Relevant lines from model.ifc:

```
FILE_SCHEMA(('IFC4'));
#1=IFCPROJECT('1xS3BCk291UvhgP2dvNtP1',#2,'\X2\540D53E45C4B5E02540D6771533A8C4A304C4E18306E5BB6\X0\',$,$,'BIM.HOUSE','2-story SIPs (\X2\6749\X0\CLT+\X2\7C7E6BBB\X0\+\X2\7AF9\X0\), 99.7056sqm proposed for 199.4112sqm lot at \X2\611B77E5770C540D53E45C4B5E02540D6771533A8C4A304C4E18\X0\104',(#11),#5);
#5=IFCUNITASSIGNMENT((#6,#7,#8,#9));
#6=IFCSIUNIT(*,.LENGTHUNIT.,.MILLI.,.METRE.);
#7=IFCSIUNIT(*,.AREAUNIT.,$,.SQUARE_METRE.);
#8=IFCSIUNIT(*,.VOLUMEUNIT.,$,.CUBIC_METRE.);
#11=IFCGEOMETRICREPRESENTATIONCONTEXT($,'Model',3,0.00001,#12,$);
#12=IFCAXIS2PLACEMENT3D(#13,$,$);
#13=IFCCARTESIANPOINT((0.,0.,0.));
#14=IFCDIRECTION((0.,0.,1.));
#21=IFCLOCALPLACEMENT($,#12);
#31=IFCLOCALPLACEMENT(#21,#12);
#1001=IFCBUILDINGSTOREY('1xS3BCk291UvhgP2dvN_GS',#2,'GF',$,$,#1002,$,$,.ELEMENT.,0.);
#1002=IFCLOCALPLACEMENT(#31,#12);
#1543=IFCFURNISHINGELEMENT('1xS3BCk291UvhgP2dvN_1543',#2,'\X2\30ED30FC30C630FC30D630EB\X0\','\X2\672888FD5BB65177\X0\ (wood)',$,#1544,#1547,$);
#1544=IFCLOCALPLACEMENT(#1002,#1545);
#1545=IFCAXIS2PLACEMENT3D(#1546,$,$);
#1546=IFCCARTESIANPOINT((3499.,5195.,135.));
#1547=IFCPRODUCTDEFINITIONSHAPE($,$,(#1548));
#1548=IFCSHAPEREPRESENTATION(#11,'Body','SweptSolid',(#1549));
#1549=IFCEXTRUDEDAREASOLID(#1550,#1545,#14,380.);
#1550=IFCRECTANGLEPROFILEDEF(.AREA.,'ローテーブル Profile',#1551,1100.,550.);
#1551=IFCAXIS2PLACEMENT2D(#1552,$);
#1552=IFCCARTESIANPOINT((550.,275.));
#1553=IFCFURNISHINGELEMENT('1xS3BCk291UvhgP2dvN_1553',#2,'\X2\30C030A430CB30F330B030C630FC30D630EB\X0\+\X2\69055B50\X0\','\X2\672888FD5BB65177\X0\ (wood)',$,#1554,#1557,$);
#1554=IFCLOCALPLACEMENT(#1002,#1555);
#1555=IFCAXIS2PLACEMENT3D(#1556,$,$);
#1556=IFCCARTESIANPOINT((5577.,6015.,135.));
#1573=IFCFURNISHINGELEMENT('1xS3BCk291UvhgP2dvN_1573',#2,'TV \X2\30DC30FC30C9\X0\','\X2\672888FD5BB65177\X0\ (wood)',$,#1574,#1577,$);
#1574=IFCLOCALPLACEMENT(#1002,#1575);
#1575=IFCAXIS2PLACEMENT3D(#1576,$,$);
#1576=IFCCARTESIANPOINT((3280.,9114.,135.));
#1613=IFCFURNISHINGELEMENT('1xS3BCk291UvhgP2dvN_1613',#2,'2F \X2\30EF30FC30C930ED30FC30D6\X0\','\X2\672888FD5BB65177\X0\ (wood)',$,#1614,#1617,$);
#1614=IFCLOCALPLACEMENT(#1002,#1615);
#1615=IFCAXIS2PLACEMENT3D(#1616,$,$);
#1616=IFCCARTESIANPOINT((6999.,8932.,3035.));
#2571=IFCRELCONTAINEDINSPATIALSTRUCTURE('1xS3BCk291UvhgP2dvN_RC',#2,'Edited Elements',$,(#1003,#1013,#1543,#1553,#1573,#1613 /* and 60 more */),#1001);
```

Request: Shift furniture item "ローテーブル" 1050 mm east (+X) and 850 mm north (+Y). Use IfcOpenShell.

```python
import ifcopenshell
import ifcopenshell.api.geometry
import ifcopenshell.util.placement

model = ifcopenshell.open("model.ifc")

item = model.by_guid("1xS3BCk291UvhgP2dvN_1543")
matrix = ifcopenshell.util.placement.get_local_placement(item.ObjectPlacement)
matrix[0, 3] += 1050.0
matrix[1, 3] += 850.0
ifcopenshell.api.geometry.edit_object_placement(model, product=item, matrix=matrix, is_si=False)

print(ifcopenshell.util.placement.get_local_placement(item.ObjectPlacement).round(3) + 0.0)

model.write("model_v2.ifc")
```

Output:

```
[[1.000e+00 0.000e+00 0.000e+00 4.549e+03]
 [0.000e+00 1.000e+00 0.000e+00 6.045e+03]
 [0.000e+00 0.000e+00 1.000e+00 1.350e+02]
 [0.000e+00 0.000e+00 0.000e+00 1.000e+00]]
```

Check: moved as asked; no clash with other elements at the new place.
